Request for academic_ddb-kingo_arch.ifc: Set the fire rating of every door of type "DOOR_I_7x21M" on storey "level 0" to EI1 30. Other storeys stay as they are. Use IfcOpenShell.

First a look at what the model holds.

```python
import ifcopenshell
import ifcopenshell.util.element

model = ifcopenshell.open("academic_ddb-kingo_arch.ifc")
print(model.schema)
storey = next(s for s in model.by_type("IfcBuildingStorey") if s.Name == "level 0")
doors = [e for e in ifcopenshell.util.element.get_decomposition(storey) if e.is_a("IfcDoor")]
seen = {}
for e in doors:
    element_type = ifcopenshell.util.element.get_type(e)
    key = (element_type.Name if element_type != e and element_type else None, ifcopenshell.util.element.get_pset(e, "Pset_DoorCommon", "FireRating"))
    seen[key] = seen.get(key, 0) + 1
for (name, value), count in sorted(seen.items(), key=str):
    print(count, "x", name, "|", value)
```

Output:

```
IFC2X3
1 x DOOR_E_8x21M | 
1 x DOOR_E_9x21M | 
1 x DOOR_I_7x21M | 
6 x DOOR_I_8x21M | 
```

```python
import ifcopenshell
import ifcopenshell.api.pset
import ifcopenshell.util.element

model = ifcopenshell.open("academic_ddb-kingo_arch.ifc")

storey = next(s for s in model.by_type("IfcBuildingStorey") if s.Name == "level 0")
doors = [e for e in ifcopenshell.util.element.get_decomposition(storey) if e.is_a("IfcDoor")]

count = 0
for e in doors:
    element_type = ifcopenshell.util.element.get_type(e)
    if element_type in (None, e) or element_type.Name != "DOOR_I_7x21M":
        continue
    # add_pset returns the element's existing set when there is one.
    pset = ifcopenshell.api.pset.add_pset(model, product=e, name="Pset_DoorCommon")
    ifcopenshell.api.pset.edit_pset(model, pset=pset, properties={"FireRating": "EI1 30"})
    count += 1

print(count, "doors updated")

model.write("academic_ddb-kingo_arch_v2.ifc")
```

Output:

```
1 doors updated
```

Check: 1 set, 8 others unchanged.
